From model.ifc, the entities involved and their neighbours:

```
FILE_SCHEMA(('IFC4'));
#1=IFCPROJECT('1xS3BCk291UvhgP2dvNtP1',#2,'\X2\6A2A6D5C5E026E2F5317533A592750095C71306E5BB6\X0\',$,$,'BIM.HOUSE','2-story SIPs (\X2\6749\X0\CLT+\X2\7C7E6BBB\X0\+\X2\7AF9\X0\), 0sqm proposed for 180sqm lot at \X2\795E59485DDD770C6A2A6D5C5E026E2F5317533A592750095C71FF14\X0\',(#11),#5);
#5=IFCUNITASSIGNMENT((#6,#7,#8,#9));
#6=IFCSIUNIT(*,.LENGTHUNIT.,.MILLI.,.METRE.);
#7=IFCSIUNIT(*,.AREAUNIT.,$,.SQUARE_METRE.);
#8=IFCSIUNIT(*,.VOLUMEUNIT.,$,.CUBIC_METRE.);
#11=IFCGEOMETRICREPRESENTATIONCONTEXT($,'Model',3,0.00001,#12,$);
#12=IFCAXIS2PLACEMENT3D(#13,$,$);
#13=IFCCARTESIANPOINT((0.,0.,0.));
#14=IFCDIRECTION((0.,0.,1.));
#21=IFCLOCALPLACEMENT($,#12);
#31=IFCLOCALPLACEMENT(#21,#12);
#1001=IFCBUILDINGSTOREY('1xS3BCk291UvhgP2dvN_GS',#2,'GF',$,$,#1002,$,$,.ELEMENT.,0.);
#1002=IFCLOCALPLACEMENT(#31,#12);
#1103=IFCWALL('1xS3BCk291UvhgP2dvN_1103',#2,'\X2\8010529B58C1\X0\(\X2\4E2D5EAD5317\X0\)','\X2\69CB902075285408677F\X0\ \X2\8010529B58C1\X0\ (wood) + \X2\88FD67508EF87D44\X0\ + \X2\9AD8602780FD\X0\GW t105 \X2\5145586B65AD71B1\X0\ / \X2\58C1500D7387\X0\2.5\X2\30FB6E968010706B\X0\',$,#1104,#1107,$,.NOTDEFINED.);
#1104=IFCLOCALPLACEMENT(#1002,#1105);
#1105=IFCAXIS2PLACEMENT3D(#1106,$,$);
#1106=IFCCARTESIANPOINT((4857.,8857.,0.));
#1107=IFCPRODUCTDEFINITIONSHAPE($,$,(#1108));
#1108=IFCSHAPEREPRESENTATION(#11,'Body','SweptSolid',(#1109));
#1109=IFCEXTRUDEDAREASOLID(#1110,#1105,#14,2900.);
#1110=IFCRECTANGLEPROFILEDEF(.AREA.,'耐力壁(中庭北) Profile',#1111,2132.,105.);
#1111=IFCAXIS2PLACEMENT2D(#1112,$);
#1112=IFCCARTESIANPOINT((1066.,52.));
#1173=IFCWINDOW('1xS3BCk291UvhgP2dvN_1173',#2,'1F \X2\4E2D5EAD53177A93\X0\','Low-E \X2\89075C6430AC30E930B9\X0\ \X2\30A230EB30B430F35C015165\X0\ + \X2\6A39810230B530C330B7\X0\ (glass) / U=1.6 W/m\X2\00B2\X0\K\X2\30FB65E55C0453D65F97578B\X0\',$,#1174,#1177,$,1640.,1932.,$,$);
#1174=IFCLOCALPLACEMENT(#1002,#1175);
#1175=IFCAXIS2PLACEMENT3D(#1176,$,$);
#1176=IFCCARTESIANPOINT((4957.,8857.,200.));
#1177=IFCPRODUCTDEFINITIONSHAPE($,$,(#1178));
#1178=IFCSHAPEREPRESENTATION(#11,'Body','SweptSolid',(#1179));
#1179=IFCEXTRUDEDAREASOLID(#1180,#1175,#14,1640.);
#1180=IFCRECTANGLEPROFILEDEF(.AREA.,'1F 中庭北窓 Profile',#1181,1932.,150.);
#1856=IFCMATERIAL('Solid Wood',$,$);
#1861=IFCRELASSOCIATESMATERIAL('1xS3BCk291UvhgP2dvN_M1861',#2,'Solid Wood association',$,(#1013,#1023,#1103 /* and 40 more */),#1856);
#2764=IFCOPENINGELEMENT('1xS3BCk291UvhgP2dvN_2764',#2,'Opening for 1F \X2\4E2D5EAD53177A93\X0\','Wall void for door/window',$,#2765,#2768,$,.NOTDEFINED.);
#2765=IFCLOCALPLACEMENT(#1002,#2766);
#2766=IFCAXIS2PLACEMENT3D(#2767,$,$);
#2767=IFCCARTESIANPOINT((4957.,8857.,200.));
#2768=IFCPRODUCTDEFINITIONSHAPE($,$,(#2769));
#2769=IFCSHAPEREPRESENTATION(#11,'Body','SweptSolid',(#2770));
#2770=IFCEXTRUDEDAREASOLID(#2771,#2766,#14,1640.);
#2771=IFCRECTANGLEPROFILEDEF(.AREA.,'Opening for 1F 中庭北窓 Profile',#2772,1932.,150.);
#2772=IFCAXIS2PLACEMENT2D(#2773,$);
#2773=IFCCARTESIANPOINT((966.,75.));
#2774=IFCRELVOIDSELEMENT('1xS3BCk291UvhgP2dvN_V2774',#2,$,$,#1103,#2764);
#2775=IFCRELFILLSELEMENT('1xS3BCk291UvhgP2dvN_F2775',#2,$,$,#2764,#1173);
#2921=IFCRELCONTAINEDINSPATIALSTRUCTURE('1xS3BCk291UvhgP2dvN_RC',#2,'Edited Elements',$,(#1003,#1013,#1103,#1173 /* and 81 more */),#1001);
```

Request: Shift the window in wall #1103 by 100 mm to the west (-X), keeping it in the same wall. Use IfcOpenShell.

```python
import ifcopenshell
import ifcopenshell.api.geometry
import ifcopenshell.util.placement
import ifcopenshell.util.unit

model = ifcopenshell.open("model.ifc")
unit_scale = ifcopenshell.util.unit.calculate_unit_scale(model)

window = model.by_guid("1xS3BCk291UvhgP2dvN_1173")
opening = window.FillsVoids[0].RelatingOpeningElement
wall = opening.VoidsElements[0].RelatingBuildingElement

wall_matrix = ifcopenshell.util.placement.get_local_placement(wall.ObjectPlacement)
shift = wall_matrix[:3, 0] * -0.1 / unit_scale
before = ifcopenshell.util.placement.get_local_placement(window.ObjectPlacement)[:3, 3].copy()

# The window is not placed relative to its opening, so move both.
for product in (opening, window):
    matrix = ifcopenshell.util.placement.get_local_placement(product.ObjectPlacement)
    matrix[:3, 3] += shift
    ifcopenshell.api.geometry.edit_object_placement(model, product=product, matrix=matrix, is_si=False)

after = ifcopenshell.util.placement.get_local_placement(window.ObjectPlacement)[:3, 3]
print("window moved by", (after - before).round(3) + 0.0)

model.write("model_rev.ifc")
```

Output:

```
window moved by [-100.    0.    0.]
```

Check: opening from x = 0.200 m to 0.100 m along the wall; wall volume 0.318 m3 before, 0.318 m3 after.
